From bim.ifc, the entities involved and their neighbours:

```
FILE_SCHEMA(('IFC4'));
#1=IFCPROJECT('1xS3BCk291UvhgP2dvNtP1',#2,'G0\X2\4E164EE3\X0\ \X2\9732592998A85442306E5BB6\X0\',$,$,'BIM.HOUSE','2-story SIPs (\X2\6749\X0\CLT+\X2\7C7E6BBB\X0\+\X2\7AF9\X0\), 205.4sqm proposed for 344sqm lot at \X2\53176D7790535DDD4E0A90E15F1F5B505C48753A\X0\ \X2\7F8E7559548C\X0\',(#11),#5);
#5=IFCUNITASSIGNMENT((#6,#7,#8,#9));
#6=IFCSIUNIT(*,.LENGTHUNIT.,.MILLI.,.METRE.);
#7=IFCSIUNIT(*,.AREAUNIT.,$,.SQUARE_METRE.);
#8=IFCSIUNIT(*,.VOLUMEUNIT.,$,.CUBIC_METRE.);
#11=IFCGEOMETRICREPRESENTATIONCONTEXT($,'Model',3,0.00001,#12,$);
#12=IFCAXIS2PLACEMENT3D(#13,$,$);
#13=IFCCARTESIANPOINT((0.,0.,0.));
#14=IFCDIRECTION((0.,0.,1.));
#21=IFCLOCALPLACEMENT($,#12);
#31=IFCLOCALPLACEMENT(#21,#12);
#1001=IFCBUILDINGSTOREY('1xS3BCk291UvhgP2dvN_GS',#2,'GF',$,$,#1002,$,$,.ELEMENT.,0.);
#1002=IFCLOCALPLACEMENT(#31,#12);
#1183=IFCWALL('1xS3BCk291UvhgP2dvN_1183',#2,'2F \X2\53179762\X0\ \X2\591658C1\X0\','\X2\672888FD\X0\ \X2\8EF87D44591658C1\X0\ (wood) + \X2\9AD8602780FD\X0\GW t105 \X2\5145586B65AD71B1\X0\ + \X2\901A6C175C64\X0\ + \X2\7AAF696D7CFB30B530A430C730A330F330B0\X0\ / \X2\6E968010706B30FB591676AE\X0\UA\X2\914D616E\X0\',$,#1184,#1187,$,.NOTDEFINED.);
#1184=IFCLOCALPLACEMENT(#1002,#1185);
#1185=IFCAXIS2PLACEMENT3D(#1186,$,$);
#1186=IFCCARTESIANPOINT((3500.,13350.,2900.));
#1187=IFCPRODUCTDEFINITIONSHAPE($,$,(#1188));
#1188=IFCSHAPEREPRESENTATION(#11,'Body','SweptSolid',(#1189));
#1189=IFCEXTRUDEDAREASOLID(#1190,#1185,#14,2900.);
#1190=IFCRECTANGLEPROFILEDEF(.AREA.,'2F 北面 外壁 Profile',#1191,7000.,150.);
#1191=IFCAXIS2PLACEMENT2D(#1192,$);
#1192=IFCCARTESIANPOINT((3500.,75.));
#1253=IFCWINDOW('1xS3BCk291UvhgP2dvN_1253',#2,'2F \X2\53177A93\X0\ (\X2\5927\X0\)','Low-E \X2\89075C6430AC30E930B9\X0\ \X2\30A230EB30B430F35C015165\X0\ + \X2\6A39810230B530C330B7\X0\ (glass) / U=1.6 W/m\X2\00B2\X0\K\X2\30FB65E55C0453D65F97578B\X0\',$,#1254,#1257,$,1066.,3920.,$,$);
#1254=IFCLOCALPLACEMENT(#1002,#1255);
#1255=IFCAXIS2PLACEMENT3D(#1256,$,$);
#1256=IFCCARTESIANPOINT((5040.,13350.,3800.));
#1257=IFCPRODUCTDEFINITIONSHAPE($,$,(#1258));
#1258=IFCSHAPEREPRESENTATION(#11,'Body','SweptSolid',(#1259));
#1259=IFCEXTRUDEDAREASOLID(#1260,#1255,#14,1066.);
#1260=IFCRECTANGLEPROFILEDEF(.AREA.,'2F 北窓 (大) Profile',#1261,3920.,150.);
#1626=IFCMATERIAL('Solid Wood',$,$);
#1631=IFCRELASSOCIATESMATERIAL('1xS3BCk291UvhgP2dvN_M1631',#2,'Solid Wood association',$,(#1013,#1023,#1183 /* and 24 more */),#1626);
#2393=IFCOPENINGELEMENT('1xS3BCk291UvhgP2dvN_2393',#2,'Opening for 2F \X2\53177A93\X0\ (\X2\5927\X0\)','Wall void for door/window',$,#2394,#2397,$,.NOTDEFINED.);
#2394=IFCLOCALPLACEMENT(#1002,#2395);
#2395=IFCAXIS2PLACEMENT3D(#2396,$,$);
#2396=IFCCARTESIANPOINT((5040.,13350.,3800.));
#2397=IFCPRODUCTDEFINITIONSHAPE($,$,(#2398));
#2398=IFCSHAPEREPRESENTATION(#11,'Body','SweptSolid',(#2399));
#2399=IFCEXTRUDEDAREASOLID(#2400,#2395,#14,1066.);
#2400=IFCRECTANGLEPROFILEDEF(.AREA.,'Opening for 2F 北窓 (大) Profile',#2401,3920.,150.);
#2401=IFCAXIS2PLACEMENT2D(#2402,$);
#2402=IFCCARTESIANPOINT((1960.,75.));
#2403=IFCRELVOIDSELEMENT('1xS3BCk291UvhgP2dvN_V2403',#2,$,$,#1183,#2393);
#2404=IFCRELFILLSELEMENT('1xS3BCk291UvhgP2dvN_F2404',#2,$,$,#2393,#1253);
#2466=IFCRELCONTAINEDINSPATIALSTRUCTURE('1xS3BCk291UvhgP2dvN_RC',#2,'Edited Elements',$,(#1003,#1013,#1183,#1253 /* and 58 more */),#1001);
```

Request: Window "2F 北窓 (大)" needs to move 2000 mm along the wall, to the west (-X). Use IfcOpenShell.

```python
import ifcopenshell
import ifcopenshell.api.geometry
import ifcopenshell.util.placement

model = ifcopenshell.open("bim.ifc")

window = model.by_guid("1xS3BCk291UvhgP2dvN_1253")
opening = window.FillsVoids[0].RelatingOpeningElement
wall = opening.VoidsElements[0].RelatingBuildingElement

wall_matrix = ifcopenshell.util.placement.get_local_placement(wall.ObjectPlacement)
shift = wall_matrix[:3, 0] * -2000.0
before = ifcopenshell.util.placement.get_local_placement(window.ObjectPlacement)[:3, 3].copy()

# The window is not placed relative to its opening, so move both.
for product in (opening, window):
    matrix = ifcopenshell.util.placement.get_local_placement(product.ObjectPlacement)
    matrix[:3, 3] += shift
    ifcopenshell.api.geometry.edit_object_placement(model, product=product, matrix=matrix, is_si=False)

after = ifcopenshell.util.placement.get_local_placement(window.ObjectPlacement)[:3, 3]
print("window moved by", (after - before).round(3) + 0.0)

model.write("bim_edited.ifc")
```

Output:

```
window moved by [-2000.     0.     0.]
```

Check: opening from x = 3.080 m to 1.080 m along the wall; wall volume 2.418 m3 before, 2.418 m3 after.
